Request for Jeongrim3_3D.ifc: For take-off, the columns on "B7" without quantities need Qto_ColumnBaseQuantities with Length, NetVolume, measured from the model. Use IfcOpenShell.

First a look at what the model holds.

```python
import ifcopenshell
import ifcopenshell.util.element
import ifcopenshell.util.unit

model = ifcopenshell.open("Jeongrim3_3D.ifc")
print(model.schema)
for unit_type in ("LENGTHUNIT", "AREAUNIT", "VOLUMEUNIT"):
    print(unit_type, ifcopenshell.util.unit.calculate_unit_scale(model, unit_type))
storey = next(s for s in model.by_type("IfcBuildingStorey") if s.Name == "B7")
columns = [e for e in ifcopenshell.util.element.get_decomposition(storey) if e.is_a("IfcColumn")]
for e in sorted(columns, key=lambda e: e.id()):
    print(e.id(), e.is_a(), e.Name, list(ifcopenshell.util.element.get_psets(e, qtos_only=True)), sep=" | ")
```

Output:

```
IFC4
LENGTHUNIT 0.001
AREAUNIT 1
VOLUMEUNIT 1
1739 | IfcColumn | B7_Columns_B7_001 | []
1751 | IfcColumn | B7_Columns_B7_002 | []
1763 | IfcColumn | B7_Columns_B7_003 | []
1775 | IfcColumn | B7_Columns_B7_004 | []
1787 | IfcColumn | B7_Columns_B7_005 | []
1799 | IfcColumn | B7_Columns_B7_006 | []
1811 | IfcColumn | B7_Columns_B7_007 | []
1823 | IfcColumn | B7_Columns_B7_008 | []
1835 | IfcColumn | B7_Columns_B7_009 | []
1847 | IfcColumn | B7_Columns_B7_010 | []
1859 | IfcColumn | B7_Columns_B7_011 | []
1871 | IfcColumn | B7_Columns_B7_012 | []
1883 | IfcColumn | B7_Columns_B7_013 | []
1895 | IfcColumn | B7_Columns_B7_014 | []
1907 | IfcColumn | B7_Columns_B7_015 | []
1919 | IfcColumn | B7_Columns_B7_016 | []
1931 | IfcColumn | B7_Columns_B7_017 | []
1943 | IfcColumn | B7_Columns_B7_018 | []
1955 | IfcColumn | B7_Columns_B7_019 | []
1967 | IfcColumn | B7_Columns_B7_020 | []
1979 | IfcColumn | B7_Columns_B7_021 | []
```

```python
import ifcopenshell
import ifcopenshell.api.pset
import ifcopenshell.geom
import ifcopenshell.util.element
import ifcopenshell.util.shape
import ifcopenshell.util.unit

model = ifcopenshell.open("Jeongrim3_3D.ifc")
unit_scale = ifcopenshell.util.unit.calculate_unit_scale(model)
volume_scale = ifcopenshell.util.unit.calculate_unit_scale(model, "VOLUMEUNIT")
settings = ifcopenshell.geom.settings()

storey = next(s for s in model.by_type("IfcBuildingStorey") if s.Name == "B7")
columns = [e for e in ifcopenshell.util.element.get_decomposition(storey) if e.is_a("IfcColumn")]

for e in sorted(columns, key=lambda e: e.id()):
    if ifcopenshell.util.element.get_psets(e, qtos_only=True, should_inherit=False):
        continue
    # Geometry comes back in metres, in the element's own axes.
    shape = ifcopenshell.geom.create_shape(settings, e)
    values = {
        "Length": ifcopenshell.util.shape.get_z(shape.geometry) / unit_scale,
        "NetVolume": ifcopenshell.util.shape.get_volume(shape.geometry) / volume_scale,
    }
    qto = ifcopenshell.api.pset.add_qto(model, product=e, name="Qto_ColumnBaseQuantities")
    ifcopenshell.api.pset.edit_qto(model, qto=qto, properties=values)
    print(e.id(), {k: round(v, 3) for k, v in values.items()})

model.write("Jeongrim3_3D_edited.ifc")
```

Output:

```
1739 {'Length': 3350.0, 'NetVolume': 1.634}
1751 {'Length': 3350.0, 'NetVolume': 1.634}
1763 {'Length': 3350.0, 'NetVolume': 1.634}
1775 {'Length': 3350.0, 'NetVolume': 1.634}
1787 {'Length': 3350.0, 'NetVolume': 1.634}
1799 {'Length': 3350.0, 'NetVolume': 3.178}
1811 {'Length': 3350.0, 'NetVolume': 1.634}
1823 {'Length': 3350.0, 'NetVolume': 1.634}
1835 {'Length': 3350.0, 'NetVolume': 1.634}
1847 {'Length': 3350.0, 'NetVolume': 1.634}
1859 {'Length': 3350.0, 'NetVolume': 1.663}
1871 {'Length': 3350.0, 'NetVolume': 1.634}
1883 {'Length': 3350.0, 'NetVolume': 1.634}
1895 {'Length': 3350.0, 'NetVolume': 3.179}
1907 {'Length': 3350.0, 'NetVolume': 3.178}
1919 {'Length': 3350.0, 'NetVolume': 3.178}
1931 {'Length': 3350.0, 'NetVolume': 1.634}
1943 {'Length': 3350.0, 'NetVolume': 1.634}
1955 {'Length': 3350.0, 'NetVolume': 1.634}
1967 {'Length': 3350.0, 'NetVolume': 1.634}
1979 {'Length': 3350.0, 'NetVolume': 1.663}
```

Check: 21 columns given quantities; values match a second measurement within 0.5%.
